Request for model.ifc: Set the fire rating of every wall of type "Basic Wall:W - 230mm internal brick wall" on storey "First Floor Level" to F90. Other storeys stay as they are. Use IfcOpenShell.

First a look at what the model holds.

```python
import ifcopenshell
import ifcopenshell.util.element

model = ifcopenshell.open("model.ifc")
print(model.schema)
storey = next(s for s in model.by_type("IfcBuildingStorey") if s.Name == "First Floor Level")
walls = [e for e in ifcopenshell.util.element.get_decomposition(storey) if e.is_a("IfcWall")]
seen = {}
for e in walls:
    element_type = ifcopenshell.util.element.get_type(e)
    key = (element_type.Name if element_type != e and element_type else None, ifcopenshell.util.element.get_pset(e, "Pset_WallCommon", "FireRating"))
    seen[key] = seen.get(key, 0) + 1
for (name, value), count in sorted(seen.items(), key=str):
    print(count, "x", name, "|", value)
```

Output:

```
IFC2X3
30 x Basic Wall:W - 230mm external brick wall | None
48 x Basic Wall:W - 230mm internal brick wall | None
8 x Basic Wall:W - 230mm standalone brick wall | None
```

```python
import ifcopenshell
import ifcopenshell.api.pset
import ifcopenshell.util.element

model = ifcopenshell.open("model.ifc")

storey = next(s for s in model.by_type("IfcBuildingStorey") if s.Name == "First Floor Level")
walls = [e for e in ifcopenshell.util.element.get_decomposition(storey) if e.is_a("IfcWall")]

count = 0
for e in walls:
    element_type = ifcopenshell.util.element.get_type(e)
    if element_type in (None, e) or element_type.Name != "Basic Wall:W - 230mm internal brick wall":
        continue
    # add_pset returns the element's existing set when there is one.
    pset = ifcopenshell.api.pset.add_pset(model, product=e, name="Pset_WallCommon")
    ifcopenshell.api.pset.edit_pset(model, pset=pset, properties={"FireRating": "F90"})
    count += 1

print(count, "walls updated")

model.write("model_v2.ifc")
```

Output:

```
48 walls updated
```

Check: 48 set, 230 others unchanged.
